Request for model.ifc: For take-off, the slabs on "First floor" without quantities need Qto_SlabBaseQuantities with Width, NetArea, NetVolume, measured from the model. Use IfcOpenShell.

First a look at what the model holds.

```python
import ifcopenshell
import ifcopenshell.util.element
import ifcopenshell.util.unit

model = ifcopenshell.open("model.ifc")
print(model.schema)
for unit_type in ("LENGTHUNIT", "AREAUNIT", "VOLUMEUNIT"):
    print(unit_type, ifcopenshell.util.unit.calculate_unit_scale(model, unit_type))
storey = next(s for s in model.by_type("IfcBuildingStorey") if s.Name == "First floor")
slabs = [e for e in ifcopenshell.util.element.get_decomposition(storey) if e.is_a("IfcSlab")]
for e in sorted(slabs, key=lambda e: e.id()):
    print(e.id(), e.is_a(), e.Name, list(ifcopenshell.util.element.get_psets(e, qtos_only=True)), sep=" | ")
```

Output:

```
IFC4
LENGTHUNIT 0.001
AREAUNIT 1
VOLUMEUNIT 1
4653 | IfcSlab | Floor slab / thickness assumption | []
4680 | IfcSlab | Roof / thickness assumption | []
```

```python
import ifcopenshell
import ifcopenshell.api.pset
import ifcopenshell.geom
import ifcopenshell.util.element
import ifcopenshell.util.shape
import ifcopenshell.util.unit

model = ifcopenshell.open("model.ifc")
unit_scale = ifcopenshell.util.unit.calculate_unit_scale(model)
area_scale = ifcopenshell.util.unit.calculate_unit_scale(model, "AREAUNIT")
volume_scale = ifcopenshell.util.unit.calculate_unit_scale(model, "VOLUMEUNIT")
settings = ifcopenshell.geom.settings()

storey = next(s for s in model.by_type("IfcBuildingStorey") if s.Name == "First floor")
slabs = [e for e in ifcopenshell.util.element.get_decomposition(storey) if e.is_a("IfcSlab")]

for e in sorted(slabs, key=lambda e: e.id()):
    if ifcopenshell.util.element.get_psets(e, qtos_only=True, should_inherit=False):
        continue
    # Geometry comes back in metres, in the element's own axes.
    shape = ifcopenshell.geom.create_shape(settings, e)
    values = {
        "Width": ifcopenshell.util.shape.get_z(shape.geometry) / unit_scale,
        "NetArea": ifcopenshell.util.shape.get_footprint_area(shape.geometry) / area_scale,
        "NetVolume": ifcopenshell.util.shape.get_volume(shape.geometry) / volume_scale,
    }
    qto = ifcopenshell.api.pset.add_qto(model, product=e, name="Qto_SlabBaseQuantities")
    ifcopenshell.api.pset.edit_qto(model, qto=qto, properties=values)
    print(e.id(), {k: round(v, 3) for k, v in values.items()})

model.write("model-out.ifc")
```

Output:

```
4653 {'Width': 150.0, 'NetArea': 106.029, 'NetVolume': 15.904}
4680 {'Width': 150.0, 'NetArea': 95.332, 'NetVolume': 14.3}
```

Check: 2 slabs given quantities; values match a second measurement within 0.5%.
